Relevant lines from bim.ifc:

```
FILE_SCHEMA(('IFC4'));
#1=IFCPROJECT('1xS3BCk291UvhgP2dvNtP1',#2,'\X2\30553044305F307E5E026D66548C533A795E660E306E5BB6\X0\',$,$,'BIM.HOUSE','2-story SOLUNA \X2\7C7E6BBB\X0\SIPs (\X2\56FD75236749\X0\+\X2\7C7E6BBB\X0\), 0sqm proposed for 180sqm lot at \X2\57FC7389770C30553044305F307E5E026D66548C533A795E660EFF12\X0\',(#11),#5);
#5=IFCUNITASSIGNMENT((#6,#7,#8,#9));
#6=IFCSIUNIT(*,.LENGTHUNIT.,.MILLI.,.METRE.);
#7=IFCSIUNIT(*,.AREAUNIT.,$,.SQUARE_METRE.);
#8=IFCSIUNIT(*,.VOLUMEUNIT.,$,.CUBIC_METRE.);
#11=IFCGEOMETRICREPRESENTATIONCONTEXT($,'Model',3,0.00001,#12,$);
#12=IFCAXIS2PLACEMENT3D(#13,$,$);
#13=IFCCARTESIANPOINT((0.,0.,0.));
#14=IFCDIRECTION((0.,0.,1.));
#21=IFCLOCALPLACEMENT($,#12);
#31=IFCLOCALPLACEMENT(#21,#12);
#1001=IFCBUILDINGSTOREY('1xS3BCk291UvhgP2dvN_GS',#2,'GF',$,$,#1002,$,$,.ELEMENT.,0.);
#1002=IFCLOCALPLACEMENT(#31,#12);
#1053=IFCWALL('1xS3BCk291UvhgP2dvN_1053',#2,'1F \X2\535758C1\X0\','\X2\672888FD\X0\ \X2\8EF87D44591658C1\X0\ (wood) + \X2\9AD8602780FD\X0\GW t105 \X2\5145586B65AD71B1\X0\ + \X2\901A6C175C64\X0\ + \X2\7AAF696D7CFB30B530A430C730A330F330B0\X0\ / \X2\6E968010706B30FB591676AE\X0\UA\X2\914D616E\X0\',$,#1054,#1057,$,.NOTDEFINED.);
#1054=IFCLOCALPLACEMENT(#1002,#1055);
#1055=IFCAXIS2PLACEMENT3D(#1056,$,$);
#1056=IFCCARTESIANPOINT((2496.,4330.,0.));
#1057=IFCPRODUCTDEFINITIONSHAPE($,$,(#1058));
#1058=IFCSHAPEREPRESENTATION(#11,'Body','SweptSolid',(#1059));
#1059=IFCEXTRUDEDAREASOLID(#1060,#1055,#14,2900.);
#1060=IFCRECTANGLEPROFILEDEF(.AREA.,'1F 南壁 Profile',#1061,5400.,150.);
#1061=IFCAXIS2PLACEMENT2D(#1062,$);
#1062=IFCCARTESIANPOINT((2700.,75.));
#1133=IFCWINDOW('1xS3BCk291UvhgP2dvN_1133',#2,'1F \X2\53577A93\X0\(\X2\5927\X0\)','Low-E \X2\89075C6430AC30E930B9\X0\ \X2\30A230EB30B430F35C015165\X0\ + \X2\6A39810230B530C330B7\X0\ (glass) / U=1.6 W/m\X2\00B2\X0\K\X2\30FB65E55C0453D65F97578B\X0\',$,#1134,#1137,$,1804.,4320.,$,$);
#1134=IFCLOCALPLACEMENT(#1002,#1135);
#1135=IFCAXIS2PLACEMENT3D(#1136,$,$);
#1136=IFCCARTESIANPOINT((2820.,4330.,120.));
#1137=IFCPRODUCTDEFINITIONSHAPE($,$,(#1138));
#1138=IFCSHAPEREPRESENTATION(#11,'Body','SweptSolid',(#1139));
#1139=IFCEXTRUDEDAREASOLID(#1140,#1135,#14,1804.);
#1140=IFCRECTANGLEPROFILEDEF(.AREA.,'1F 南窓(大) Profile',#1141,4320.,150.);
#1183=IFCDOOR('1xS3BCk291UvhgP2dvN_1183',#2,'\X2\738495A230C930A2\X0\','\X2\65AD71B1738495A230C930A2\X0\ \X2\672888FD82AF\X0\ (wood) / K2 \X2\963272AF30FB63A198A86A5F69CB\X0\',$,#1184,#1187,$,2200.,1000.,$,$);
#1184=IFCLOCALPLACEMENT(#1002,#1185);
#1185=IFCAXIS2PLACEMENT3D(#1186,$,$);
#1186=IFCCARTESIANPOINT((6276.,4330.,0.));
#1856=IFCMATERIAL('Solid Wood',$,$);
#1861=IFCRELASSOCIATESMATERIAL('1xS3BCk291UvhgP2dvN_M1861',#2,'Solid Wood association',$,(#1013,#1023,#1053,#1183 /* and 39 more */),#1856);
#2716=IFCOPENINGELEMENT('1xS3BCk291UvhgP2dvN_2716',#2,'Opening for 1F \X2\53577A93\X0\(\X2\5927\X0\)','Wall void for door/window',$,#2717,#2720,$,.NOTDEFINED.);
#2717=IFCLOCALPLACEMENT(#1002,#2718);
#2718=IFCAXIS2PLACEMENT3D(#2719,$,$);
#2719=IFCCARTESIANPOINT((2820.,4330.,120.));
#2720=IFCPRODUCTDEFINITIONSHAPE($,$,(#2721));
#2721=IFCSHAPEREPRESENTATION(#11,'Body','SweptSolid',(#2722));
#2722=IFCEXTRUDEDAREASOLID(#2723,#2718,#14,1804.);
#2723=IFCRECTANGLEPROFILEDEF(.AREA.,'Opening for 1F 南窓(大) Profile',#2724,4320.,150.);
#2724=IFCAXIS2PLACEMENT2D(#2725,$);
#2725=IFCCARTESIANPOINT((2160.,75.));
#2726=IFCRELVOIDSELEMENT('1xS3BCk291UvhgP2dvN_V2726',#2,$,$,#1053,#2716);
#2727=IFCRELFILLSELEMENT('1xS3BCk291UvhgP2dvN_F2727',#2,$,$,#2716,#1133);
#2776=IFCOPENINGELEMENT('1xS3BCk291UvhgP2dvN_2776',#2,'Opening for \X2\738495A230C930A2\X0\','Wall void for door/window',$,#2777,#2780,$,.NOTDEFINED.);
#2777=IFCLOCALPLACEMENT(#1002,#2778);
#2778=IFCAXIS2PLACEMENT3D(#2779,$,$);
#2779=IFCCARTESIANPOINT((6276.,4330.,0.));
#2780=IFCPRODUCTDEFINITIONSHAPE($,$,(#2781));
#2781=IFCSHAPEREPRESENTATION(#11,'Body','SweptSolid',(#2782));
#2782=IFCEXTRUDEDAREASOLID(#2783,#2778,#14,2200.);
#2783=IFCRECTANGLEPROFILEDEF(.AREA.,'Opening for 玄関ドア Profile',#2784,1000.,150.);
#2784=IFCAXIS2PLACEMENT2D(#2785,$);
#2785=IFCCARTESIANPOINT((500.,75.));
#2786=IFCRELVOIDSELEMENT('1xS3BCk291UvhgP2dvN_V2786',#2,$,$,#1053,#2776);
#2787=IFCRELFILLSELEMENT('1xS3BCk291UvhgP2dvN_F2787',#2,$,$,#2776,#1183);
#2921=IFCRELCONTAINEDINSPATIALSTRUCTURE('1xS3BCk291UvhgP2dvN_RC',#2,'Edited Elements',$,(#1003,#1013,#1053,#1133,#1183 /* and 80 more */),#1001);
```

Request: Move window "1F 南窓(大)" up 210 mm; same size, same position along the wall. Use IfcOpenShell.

```python
import numpy as np
import ifcopenshell
import ifcopenshell.api.geometry
import ifcopenshell.util.placement
import ifcopenshell.util.unit

model = ifcopenshell.open("bim.ifc")
unit_scale = ifcopenshell.util.unit.calculate_unit_scale(model)

window = model.by_guid("1xS3BCk291UvhgP2dvN_1133")
opening = window.FillsVoids[0].RelatingOpeningElement
dz = 210.0

shift = np.array([0.0, 0.0, dz])
# The window is not placed relative to its opening, so move both.
for product in (opening, window):
    matrix = ifcopenshell.util.placement.get_local_placement(product.ObjectPlacement)
    matrix[:3, 3] += shift
    ifcopenshell.api.geometry.edit_object_placement(model, product=product, matrix=matrix, is_si=False)

print(f"moved by {dz * unit_scale:+.3f} m")

model.write("bim_edited.ifc")
```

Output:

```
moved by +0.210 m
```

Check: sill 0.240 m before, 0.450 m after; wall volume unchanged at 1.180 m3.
